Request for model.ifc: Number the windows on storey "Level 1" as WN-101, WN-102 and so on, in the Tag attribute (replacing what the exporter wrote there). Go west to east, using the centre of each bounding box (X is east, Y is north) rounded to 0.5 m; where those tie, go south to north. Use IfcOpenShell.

First a look at what the model holds.

```python
import ifcopenshell
import ifcopenshell.util.element
import ifcopenshell.util.placement

model = ifcopenshell.open("model.ifc")
print(model.schema)
storey = next(s for s in model.by_type("IfcBuildingStorey") if s.Name == "Level 1")
windows = [e for e in ifcopenshell.util.element.get_decomposition(storey) if e.is_a("IfcWindow")]
for e in sorted(windows, key=lambda e: e.id()):
    origin = ifcopenshell.util.placement.get_local_placement(e.ObjectPlacement)[:3, 3]
    print(e.id(), e.Tag, e.Name, origin.round(2) + 0.0, sep=" | ")
```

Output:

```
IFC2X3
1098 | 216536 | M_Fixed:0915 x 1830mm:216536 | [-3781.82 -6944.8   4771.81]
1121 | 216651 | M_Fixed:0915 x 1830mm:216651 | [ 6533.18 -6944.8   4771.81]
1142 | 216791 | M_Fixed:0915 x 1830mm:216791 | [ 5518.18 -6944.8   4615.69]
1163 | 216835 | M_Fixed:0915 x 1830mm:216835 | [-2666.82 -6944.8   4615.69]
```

```python
import ifcopenshell
import ifcopenshell.geom
import ifcopenshell.util.element
import ifcopenshell.util.shape

model = ifcopenshell.open("model.ifc")
settings = ifcopenshell.geom.settings()
settings.set("use-world-coords", True)


def centre(element):
    shape = ifcopenshell.geom.create_shape(settings, element)
    return ifcopenshell.util.shape.get_bbox_centroid(shape.geometry)


storey = next(s for s in model.by_type("IfcBuildingStorey") if s.Name == "Level 1")
windows = [e for e in ifcopenshell.util.element.get_decomposition(storey) if e.is_a("IfcWindow")]

# Insertion points can sit at a corner or the storey origin, so sort by the geometry (in metres).
centres = {e: centre(e) for e in windows}
windows.sort(key=lambda e: (round(centres[e][0] / 0.5), centres[e][1]))

for i, e in enumerate(windows, start=1):
    number = f"WN-1{i:02d}"
    e.Tag = number
    print(e.id(), number)

model.write("model-out.ifc")
```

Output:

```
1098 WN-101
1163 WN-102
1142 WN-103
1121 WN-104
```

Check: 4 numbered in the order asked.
